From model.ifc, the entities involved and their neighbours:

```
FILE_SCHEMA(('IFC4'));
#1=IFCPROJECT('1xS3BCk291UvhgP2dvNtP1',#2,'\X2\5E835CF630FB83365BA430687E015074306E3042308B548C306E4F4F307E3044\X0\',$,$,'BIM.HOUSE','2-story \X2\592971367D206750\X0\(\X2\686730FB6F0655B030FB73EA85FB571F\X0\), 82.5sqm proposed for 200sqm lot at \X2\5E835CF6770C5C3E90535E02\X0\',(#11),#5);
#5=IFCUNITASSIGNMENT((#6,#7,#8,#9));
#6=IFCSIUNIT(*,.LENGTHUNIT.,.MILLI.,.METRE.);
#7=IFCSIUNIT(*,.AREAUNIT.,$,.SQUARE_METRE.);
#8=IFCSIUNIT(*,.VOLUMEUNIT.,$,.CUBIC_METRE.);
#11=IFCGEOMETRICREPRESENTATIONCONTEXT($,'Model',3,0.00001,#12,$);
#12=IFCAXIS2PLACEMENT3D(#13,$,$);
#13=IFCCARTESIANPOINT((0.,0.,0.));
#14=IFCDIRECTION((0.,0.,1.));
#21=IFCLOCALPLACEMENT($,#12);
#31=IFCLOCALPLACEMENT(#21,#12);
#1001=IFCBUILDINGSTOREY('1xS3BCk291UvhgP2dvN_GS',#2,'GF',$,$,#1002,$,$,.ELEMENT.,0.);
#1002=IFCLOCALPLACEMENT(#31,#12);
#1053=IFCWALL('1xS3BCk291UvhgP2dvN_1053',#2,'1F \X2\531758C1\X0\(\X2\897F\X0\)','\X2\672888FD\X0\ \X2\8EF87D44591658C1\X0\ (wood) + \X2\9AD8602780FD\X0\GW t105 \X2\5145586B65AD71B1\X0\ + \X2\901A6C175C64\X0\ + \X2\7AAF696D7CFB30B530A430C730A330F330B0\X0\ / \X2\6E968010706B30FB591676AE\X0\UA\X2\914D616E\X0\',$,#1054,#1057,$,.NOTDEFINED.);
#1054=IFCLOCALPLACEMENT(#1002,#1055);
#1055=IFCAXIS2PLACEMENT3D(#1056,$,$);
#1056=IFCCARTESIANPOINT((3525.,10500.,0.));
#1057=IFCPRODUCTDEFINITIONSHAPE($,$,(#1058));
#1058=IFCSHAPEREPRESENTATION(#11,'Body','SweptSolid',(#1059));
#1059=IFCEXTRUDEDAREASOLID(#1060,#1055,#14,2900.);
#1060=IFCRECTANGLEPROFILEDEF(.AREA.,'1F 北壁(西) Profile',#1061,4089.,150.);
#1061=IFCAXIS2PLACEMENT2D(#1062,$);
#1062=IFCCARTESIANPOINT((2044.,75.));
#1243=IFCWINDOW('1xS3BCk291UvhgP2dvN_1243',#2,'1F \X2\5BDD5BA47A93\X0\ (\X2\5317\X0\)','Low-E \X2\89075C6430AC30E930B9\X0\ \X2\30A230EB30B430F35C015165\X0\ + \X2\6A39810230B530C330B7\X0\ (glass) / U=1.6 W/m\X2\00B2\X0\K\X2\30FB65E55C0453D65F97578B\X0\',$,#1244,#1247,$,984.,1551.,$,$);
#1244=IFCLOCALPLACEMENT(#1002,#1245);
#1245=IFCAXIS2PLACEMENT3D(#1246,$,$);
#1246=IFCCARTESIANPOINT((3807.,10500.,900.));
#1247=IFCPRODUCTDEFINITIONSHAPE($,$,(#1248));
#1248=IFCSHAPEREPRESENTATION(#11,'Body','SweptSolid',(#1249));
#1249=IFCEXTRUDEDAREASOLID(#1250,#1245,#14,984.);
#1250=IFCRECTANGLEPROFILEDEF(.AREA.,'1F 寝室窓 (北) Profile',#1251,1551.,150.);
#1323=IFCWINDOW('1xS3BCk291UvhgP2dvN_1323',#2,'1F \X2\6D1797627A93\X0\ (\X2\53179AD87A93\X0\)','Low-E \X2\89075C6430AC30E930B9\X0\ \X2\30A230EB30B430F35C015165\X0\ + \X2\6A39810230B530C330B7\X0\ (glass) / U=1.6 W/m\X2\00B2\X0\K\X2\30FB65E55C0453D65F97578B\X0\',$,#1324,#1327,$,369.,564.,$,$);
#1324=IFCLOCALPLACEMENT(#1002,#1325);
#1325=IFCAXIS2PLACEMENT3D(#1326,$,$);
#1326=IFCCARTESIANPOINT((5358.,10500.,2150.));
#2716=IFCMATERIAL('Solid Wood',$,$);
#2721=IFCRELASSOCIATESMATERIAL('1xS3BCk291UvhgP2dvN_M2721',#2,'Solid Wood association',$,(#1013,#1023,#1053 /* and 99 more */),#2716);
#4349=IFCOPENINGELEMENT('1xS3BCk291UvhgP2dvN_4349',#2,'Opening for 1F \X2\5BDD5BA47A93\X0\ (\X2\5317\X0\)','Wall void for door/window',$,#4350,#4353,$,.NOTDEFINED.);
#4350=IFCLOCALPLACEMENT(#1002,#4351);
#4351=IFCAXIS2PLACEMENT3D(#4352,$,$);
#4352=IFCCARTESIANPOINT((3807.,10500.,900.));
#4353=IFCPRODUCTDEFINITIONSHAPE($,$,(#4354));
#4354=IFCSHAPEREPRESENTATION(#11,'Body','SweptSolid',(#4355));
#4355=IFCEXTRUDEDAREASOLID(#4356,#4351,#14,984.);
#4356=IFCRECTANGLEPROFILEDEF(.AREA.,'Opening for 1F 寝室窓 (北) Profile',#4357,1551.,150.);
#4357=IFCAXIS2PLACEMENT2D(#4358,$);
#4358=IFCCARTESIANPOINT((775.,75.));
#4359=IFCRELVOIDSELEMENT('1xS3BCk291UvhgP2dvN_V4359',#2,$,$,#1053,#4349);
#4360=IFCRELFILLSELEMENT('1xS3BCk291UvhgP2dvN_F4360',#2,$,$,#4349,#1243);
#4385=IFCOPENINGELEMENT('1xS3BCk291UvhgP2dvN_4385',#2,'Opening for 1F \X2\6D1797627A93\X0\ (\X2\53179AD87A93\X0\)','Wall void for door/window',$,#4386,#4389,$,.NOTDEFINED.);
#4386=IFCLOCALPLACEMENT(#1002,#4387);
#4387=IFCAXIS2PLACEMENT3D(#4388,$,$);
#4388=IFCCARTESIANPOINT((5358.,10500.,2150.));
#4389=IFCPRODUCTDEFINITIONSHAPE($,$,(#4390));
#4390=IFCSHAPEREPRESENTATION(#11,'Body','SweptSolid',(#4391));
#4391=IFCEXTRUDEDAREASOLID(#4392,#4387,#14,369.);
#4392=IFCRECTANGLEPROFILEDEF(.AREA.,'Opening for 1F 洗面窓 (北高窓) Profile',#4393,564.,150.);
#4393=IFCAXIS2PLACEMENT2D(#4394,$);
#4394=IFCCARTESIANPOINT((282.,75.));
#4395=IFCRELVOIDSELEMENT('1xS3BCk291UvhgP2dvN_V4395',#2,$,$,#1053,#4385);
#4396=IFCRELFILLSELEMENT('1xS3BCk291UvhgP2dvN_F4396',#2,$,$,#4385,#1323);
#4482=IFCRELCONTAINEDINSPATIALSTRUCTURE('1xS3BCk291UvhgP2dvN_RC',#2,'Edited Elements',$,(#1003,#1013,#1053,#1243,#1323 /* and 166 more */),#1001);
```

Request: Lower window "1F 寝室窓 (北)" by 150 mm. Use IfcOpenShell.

```python
import numpy as np
import ifcopenshell
import ifcopenshell.api.geometry
import ifcopenshell.util.placement
import ifcopenshell.util.unit

model = ifcopenshell.open("model.ifc")
unit_scale = ifcopenshell.util.unit.calculate_unit_scale(model)

window = model.by_id(1243)
opening = window.FillsVoids[0].RelatingOpeningElement
dz = -0.15 / unit_scale

shift = np.array([0.0, 0.0, dz])
# The window is not placed relative to its opening, so move both.
for product in (opening, window):
    matrix = ifcopenshell.util.placement.get_local_placement(product.ObjectPlacement)
    matrix[:3, 3] += shift
    ifcopenshell.api.geometry.edit_object_placement(model, product=product, matrix=matrix, is_si=False)

print(f"moved by {dz * unit_scale:+.3f} m")

model.write("model_updated.ifc")
```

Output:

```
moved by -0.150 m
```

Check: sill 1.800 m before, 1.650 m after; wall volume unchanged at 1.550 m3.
